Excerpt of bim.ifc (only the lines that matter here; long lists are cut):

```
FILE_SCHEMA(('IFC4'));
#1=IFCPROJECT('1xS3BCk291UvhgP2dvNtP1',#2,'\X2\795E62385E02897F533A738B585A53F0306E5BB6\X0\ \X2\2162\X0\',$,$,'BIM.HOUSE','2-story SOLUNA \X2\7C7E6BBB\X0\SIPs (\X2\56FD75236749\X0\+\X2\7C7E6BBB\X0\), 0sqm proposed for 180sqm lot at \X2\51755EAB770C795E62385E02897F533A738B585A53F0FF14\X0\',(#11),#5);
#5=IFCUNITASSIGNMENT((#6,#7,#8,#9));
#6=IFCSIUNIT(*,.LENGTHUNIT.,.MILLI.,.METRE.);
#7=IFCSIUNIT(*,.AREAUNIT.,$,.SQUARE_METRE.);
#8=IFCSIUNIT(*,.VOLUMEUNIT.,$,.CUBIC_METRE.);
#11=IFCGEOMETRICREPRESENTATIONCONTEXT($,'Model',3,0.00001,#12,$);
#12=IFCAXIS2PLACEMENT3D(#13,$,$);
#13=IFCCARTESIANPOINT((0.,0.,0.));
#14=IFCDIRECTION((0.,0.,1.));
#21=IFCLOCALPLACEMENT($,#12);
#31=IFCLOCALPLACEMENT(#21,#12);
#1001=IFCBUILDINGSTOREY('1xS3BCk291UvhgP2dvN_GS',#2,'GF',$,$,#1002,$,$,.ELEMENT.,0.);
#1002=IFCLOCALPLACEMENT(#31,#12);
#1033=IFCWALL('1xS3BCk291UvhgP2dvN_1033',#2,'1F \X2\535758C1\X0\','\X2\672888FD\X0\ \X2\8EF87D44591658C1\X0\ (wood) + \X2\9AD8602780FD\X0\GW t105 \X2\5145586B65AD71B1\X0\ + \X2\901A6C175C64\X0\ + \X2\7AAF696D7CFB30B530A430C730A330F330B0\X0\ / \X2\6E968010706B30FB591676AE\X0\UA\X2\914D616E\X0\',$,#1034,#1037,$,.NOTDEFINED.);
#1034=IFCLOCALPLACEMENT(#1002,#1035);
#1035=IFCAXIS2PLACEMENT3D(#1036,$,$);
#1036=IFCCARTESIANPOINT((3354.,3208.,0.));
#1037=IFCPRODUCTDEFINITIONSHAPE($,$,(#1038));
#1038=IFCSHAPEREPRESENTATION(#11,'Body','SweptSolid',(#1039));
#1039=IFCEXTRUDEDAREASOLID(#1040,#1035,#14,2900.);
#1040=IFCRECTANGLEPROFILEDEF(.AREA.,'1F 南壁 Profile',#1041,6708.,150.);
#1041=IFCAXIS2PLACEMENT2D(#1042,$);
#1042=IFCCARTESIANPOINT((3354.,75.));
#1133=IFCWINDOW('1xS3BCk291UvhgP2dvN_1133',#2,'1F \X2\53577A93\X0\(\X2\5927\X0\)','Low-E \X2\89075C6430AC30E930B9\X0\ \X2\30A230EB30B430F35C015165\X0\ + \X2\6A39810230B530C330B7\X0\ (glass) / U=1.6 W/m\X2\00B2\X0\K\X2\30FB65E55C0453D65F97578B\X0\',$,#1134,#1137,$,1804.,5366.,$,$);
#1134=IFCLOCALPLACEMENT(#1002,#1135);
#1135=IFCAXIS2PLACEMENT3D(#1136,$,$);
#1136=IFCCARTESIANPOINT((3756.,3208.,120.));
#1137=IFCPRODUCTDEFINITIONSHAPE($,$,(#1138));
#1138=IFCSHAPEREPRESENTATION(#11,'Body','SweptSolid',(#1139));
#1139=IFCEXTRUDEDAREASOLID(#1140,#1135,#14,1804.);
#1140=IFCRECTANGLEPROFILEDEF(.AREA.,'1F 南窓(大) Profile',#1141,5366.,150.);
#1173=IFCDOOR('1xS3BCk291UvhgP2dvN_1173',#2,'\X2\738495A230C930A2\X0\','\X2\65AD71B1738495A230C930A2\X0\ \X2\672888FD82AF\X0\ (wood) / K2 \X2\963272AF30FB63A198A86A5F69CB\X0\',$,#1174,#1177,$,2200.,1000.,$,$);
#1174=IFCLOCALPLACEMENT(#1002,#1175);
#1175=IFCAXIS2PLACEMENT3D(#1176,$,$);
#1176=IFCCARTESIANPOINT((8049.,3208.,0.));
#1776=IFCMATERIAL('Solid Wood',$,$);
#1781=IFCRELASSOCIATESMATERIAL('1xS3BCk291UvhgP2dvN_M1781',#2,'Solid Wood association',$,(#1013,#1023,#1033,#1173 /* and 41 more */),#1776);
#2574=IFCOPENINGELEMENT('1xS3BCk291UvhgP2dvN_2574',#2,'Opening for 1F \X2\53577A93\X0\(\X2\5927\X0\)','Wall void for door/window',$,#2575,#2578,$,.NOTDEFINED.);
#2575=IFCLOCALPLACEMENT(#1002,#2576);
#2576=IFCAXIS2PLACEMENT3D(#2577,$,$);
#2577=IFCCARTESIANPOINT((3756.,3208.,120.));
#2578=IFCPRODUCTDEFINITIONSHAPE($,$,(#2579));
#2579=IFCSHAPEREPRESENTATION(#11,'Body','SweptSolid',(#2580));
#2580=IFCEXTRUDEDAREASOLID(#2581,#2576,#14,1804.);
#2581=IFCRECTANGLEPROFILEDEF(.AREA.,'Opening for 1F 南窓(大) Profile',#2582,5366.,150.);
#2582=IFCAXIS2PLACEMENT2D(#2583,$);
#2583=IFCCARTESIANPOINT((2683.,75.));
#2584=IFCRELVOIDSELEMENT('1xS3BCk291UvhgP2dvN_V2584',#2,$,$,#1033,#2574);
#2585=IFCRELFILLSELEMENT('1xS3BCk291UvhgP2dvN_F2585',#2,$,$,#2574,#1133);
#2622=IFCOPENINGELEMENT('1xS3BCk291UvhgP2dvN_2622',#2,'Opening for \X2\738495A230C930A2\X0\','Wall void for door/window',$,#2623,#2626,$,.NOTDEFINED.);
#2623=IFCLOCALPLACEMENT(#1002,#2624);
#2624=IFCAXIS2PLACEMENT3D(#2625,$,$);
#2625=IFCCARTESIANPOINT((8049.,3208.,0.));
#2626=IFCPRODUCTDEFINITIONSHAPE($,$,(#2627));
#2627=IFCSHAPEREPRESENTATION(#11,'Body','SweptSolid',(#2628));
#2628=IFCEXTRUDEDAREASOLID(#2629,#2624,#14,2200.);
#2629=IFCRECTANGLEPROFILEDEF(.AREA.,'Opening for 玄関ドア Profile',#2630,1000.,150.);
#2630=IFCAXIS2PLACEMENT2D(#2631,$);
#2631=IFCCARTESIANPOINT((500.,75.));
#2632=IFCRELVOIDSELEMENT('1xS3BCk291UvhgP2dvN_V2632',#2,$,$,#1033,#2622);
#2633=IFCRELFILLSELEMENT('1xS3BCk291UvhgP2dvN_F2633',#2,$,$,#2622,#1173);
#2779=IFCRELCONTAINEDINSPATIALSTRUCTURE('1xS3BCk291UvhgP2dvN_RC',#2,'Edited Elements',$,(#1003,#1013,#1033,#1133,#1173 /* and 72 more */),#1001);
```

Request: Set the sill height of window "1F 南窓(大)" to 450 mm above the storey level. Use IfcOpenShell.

```python
import numpy as np
import ifcopenshell
import ifcopenshell.api.geometry
import ifcopenshell.geom
import ifcopenshell.util.element
import ifcopenshell.util.placement
import ifcopenshell.util.shape
import ifcopenshell.util.unit

model = ifcopenshell.open("bim.ifc")
unit_scale = ifcopenshell.util.unit.calculate_unit_scale(model)

window = model.by_guid("1xS3BCk291UvhgP2dvN_1133")
opening = window.FillsVoids[0].RelatingOpeningElement
storey = ifcopenshell.util.element.get_container(window, ifc_class="IfcBuildingStorey")
level = ifcopenshell.util.placement.get_local_placement(storey.ObjectPlacement)[2, 3]

# The opening's origin need not be at the sill, so measure its lowest point.
shape = ifcopenshell.geom.create_shape(ifcopenshell.geom.settings(), opening)
bottom = ifcopenshell.util.shape.get_shape_bottom_elevation(shape, shape.geometry) / unit_scale
dz = level + 0.45 / unit_scale - bottom

shift = np.array([0.0, 0.0, dz])
# The window is not placed relative to its opening, so move both.
for product in (opening, window):
    matrix = ifcopenshell.util.placement.get_local_placement(product.ObjectPlacement)
    matrix[:3, 3] += shift
    ifcopenshell.api.geometry.edit_object_placement(model, product=product, matrix=matrix, is_si=False)

print(f"moved by {dz * unit_scale:+.3f} m")

model.write("bim_v2.ifc")
```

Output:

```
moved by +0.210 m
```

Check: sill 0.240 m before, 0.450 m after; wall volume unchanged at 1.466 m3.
